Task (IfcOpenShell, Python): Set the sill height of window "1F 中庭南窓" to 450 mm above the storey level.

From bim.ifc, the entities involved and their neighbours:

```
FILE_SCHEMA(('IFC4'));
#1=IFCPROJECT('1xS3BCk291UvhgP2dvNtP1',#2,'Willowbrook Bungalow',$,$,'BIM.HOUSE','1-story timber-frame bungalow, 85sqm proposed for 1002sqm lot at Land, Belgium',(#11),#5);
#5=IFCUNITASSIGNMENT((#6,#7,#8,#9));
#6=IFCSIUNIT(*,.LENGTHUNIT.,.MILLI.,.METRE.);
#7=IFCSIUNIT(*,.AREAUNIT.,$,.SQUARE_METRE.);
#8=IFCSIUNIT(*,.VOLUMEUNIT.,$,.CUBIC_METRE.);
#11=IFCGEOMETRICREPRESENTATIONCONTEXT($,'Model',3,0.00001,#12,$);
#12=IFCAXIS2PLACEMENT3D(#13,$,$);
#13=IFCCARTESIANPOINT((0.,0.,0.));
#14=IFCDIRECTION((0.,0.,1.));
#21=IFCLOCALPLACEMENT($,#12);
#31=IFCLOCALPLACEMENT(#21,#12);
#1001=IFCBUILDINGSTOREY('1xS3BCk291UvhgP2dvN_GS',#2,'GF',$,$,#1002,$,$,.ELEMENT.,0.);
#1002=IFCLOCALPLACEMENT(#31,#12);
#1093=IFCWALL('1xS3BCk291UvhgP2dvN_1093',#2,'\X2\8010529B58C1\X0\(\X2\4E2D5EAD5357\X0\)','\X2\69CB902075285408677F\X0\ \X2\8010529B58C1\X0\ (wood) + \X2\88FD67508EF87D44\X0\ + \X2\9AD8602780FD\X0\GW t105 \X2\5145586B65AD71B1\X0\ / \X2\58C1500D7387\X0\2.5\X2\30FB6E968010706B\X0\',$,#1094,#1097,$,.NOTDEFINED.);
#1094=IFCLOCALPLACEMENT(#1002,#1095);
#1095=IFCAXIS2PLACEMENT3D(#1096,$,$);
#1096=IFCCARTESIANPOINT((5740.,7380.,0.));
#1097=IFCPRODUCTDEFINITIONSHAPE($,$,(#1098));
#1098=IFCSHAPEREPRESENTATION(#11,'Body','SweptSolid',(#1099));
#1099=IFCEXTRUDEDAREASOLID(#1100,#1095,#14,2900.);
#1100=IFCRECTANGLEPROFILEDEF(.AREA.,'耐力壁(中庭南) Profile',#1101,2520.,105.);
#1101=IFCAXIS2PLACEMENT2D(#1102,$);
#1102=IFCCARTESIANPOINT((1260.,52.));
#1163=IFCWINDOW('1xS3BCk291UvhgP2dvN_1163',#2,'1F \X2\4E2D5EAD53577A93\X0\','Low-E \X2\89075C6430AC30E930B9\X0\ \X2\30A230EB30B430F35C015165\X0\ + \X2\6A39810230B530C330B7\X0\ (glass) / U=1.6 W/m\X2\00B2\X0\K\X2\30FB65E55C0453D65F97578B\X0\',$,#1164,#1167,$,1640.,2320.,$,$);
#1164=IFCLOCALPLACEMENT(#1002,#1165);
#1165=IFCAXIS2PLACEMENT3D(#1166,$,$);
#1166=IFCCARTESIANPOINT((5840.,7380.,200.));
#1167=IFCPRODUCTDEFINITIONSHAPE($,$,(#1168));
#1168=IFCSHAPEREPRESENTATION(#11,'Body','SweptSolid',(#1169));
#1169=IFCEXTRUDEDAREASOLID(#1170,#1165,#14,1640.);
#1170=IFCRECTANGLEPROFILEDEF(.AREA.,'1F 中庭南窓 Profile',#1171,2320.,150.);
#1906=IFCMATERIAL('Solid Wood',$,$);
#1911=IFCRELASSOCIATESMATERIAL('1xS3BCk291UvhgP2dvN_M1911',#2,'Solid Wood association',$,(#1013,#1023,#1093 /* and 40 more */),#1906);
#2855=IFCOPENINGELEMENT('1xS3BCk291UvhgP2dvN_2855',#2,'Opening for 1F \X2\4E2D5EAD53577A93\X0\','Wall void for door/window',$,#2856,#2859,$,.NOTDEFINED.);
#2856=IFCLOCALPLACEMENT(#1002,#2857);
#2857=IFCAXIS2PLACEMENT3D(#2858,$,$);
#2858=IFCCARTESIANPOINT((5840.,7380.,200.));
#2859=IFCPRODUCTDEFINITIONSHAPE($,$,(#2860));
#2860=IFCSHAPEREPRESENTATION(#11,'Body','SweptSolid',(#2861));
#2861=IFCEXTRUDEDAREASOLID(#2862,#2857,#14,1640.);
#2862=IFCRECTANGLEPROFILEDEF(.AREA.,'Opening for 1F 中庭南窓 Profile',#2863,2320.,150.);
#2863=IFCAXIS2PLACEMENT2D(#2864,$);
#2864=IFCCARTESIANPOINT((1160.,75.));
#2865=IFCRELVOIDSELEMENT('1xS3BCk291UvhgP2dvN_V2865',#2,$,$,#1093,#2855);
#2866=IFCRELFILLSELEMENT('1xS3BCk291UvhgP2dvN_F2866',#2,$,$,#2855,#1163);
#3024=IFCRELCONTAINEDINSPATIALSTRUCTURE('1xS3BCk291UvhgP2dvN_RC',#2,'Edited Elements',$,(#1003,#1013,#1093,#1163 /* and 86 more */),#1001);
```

```python
import numpy as np
import ifcopenshell
import ifcopenshell.api.geometry
import ifcopenshell.geom
import ifcopenshell.util.element
import ifcopenshell.util.placement
import ifcopenshell.util.shape
import ifcopenshell.util.unit

model = ifcopenshell.open("bim.ifc")
unit_scale = ifcopenshell.util.unit.calculate_unit_scale(model)

window = model.by_guid("1xS3BCk291UvhgP2dvN_1163")
opening = window.FillsVoids[0].RelatingOpeningElement
storey = ifcopenshell.util.element.get_container(window, ifc_class="IfcBuildingStorey")
level = ifcopenshell.util.placement.get_local_placement(storey.ObjectPlacement)[2, 3]

# The opening's origin need not be at the sill, so measure its lowest point.
shape = ifcopenshell.geom.create_shape(ifcopenshell.geom.settings(), opening)
bottom = ifcopenshell.util.shape.get_shape_bottom_elevation(shape, shape.geometry) / unit_scale
dz = level + 450.0 - bottom

shift = np.array([0.0, 0.0, dz])
# The window is not placed relative to its opening, so move both.
for product in (opening, window):
    matrix = ifcopenshell.util.placement.get_local_placement(product.ObjectPlacement)
    matrix[:3, 3] += shift
    ifcopenshell.api.geometry.edit_object_placement(model, product=product, matrix=matrix, is_si=False)

print(f"moved by {dz * unit_scale:+.3f} m")

model.write("bim_rev.ifc")
```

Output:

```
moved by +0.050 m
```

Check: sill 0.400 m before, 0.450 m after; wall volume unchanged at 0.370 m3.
